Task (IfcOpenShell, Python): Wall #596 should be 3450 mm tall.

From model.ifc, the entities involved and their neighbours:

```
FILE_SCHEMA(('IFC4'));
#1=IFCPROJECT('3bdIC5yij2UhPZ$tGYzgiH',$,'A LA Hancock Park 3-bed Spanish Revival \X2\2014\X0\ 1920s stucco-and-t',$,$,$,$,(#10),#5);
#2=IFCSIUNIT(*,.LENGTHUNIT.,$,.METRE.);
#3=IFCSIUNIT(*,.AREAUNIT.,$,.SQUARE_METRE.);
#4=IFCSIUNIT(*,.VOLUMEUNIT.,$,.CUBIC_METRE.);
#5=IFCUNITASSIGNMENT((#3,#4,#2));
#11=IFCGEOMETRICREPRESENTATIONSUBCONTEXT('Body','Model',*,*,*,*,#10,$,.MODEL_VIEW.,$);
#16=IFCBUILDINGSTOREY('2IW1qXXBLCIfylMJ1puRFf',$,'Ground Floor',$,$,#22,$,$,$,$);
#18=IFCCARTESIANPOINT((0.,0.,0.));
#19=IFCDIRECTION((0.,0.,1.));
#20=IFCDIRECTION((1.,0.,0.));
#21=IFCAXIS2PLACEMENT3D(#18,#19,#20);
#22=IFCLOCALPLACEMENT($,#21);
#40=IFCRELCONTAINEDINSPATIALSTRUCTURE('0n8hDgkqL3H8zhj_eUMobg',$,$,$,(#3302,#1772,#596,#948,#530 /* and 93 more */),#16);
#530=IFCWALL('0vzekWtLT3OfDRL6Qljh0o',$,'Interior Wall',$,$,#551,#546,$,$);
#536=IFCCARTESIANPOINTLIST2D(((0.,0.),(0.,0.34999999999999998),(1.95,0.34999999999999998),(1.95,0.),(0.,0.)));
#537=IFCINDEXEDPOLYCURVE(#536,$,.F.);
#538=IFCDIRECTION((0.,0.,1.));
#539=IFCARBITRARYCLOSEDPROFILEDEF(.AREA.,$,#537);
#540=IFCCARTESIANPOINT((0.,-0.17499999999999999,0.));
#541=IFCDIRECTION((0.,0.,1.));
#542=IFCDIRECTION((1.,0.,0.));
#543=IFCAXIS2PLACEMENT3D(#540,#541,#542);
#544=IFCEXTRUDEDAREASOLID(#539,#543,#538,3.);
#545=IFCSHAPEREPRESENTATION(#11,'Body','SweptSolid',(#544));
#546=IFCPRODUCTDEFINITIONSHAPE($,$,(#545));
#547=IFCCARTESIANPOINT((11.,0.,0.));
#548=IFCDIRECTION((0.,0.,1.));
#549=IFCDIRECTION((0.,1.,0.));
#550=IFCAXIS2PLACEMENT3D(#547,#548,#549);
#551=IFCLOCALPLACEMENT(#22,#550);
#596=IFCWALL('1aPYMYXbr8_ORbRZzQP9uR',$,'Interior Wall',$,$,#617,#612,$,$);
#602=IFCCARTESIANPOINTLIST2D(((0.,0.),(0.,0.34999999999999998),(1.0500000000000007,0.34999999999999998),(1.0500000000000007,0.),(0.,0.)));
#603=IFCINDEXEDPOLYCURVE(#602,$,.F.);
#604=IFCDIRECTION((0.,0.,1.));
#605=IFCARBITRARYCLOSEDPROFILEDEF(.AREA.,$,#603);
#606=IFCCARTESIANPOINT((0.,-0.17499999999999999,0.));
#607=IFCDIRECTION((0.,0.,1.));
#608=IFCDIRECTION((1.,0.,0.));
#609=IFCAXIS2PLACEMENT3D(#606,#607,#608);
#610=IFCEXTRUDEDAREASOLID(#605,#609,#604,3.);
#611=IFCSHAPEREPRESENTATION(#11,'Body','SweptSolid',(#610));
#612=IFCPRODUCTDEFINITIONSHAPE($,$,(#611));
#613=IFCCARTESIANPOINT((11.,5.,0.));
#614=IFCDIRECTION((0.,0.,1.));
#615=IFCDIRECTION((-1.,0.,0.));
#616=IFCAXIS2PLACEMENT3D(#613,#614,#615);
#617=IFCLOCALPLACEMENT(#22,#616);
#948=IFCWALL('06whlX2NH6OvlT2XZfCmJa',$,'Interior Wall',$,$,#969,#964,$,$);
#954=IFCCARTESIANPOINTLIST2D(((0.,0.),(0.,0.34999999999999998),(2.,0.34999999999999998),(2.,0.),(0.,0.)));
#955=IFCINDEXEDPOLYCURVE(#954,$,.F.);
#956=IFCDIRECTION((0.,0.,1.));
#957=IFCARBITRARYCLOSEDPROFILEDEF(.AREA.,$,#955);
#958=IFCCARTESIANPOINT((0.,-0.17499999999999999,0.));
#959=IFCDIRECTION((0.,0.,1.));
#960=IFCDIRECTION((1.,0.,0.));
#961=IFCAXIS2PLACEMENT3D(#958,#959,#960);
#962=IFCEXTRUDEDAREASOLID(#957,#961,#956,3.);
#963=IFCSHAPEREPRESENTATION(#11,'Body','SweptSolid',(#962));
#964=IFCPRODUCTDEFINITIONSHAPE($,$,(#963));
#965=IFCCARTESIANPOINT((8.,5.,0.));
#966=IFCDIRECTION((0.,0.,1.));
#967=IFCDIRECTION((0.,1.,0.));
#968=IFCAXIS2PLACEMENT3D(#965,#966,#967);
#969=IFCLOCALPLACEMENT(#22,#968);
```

```python
import ifcopenshell
import ifcopenshell.geom
import ifcopenshell.util.representation
import ifcopenshell.util.shape

model = ifcopenshell.open("model.ifc")
settings = ifcopenshell.geom.settings()


def volume(element):
    """Net volume in cubic metres, openings subtracted."""
    shape = ifcopenshell.geom.create_shape(settings, element)
    return ifcopenshell.util.shape.get_volume(shape.geometry)


wall = model.by_guid("1aPYMYXbr8_ORbRZzQP9uR")
before = volume(wall)

body = ifcopenshell.util.representation.get_representation(wall, "Model", "Body")
solid = body.Items[0]
old_height = solid.Depth
solid.Depth = 3.45
after = volume(wall)

print(f"height {old_height:g} -> {solid.Depth:g}, volume {before:.3f} -> {after:.3f} m3")

model.write("model_v2.ifc")
```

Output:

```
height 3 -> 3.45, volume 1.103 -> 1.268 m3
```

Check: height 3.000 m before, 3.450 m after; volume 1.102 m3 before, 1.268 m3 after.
